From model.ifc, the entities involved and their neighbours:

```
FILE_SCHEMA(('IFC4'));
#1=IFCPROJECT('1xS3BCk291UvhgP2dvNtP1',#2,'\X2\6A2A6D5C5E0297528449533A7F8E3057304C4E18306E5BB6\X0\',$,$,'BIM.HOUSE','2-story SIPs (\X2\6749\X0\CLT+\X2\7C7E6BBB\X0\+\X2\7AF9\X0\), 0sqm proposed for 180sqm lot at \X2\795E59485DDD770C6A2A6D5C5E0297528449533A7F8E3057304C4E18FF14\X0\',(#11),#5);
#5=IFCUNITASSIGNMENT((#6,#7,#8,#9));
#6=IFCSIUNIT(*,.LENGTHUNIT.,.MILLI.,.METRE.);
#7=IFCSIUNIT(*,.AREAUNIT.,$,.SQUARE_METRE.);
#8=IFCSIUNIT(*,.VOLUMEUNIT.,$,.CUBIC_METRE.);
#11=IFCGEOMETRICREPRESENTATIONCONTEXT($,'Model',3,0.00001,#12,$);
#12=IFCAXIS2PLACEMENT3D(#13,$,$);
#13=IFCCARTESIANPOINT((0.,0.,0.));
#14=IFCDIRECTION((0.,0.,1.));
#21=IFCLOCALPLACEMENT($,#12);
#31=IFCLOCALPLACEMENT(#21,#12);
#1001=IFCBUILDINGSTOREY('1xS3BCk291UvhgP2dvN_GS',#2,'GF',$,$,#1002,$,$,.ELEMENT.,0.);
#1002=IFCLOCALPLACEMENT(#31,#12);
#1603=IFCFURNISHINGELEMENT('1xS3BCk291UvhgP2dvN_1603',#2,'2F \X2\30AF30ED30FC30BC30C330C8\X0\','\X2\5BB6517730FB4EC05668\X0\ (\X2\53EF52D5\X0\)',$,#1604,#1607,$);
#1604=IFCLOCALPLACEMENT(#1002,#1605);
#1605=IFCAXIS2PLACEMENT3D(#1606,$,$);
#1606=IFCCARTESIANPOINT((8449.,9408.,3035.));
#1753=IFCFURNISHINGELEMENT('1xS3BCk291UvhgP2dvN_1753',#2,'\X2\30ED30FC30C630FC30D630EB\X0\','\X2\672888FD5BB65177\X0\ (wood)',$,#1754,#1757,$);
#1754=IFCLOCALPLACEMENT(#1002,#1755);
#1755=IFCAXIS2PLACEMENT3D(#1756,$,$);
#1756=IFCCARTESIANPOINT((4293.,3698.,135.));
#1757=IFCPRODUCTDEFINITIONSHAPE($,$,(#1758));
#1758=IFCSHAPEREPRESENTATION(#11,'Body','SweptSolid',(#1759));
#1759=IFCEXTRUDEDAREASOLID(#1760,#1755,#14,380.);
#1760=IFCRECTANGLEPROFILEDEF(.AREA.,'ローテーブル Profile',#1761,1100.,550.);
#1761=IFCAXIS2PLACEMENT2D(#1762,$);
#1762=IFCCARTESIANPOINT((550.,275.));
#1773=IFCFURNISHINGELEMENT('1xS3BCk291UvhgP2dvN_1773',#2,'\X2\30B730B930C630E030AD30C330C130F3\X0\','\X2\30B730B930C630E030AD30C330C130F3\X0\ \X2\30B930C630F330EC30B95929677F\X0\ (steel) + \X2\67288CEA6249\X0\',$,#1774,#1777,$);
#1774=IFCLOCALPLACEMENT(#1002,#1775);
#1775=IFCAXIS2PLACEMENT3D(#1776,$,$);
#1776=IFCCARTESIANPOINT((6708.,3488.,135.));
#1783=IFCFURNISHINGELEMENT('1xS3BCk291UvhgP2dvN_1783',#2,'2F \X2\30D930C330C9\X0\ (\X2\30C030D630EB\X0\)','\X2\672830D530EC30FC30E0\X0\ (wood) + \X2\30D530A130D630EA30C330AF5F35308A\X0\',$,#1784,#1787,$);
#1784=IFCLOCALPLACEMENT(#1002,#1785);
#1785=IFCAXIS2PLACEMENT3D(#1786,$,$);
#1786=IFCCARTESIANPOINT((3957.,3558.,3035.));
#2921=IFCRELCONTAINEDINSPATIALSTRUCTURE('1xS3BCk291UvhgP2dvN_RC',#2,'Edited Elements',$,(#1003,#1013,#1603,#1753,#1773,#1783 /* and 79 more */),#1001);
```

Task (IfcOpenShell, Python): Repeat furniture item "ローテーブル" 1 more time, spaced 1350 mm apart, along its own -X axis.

```python
import ifcopenshell
import ifcopenshell.api.geometry
import ifcopenshell.api.root
import ifcopenshell.util.element
import ifcopenshell.util.placement

model = ifcopenshell.open("model.ifc")


def reuse_history(source, copy):
    """copy_class also copies each property set's owner history, people and application; keep the originals."""
    for rel in copy.IsDefinedBy:
        if rel.is_a("IfcRelDefinesByProperties") and (history := rel.RelatingPropertyDefinition.OwnerHistory):
            rel.RelatingPropertyDefinition.OwnerHistory = source.OwnerHistory
            ifcopenshell.util.element.remove_deep2(model, history)


source = model.by_id(1753)
base = ifcopenshell.util.placement.get_local_placement(source.ObjectPlacement)
step = -base[:3, 0] * 1350.0

for i in range(1, 2):
    copy = ifcopenshell.api.root.copy_class(model, product=source)
    copy.Representation = ifcopenshell.util.element.copy_deep(
        model, source.Representation, exclude=["IfcGeometricRepresentationContext", "IfcRepresentationMap"]
    )
    reuse_history(source, copy)
    matrix = base.copy()
    matrix[:3, 3] += i * step
    print("added at", matrix[:3, 3].round(3) + 0.0)
    ifcopenshell.api.geometry.edit_object_placement(model, product=copy, matrix=matrix, is_si=False)

model.write("model_edited.ifc")
```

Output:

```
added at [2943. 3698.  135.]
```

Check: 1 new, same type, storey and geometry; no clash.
